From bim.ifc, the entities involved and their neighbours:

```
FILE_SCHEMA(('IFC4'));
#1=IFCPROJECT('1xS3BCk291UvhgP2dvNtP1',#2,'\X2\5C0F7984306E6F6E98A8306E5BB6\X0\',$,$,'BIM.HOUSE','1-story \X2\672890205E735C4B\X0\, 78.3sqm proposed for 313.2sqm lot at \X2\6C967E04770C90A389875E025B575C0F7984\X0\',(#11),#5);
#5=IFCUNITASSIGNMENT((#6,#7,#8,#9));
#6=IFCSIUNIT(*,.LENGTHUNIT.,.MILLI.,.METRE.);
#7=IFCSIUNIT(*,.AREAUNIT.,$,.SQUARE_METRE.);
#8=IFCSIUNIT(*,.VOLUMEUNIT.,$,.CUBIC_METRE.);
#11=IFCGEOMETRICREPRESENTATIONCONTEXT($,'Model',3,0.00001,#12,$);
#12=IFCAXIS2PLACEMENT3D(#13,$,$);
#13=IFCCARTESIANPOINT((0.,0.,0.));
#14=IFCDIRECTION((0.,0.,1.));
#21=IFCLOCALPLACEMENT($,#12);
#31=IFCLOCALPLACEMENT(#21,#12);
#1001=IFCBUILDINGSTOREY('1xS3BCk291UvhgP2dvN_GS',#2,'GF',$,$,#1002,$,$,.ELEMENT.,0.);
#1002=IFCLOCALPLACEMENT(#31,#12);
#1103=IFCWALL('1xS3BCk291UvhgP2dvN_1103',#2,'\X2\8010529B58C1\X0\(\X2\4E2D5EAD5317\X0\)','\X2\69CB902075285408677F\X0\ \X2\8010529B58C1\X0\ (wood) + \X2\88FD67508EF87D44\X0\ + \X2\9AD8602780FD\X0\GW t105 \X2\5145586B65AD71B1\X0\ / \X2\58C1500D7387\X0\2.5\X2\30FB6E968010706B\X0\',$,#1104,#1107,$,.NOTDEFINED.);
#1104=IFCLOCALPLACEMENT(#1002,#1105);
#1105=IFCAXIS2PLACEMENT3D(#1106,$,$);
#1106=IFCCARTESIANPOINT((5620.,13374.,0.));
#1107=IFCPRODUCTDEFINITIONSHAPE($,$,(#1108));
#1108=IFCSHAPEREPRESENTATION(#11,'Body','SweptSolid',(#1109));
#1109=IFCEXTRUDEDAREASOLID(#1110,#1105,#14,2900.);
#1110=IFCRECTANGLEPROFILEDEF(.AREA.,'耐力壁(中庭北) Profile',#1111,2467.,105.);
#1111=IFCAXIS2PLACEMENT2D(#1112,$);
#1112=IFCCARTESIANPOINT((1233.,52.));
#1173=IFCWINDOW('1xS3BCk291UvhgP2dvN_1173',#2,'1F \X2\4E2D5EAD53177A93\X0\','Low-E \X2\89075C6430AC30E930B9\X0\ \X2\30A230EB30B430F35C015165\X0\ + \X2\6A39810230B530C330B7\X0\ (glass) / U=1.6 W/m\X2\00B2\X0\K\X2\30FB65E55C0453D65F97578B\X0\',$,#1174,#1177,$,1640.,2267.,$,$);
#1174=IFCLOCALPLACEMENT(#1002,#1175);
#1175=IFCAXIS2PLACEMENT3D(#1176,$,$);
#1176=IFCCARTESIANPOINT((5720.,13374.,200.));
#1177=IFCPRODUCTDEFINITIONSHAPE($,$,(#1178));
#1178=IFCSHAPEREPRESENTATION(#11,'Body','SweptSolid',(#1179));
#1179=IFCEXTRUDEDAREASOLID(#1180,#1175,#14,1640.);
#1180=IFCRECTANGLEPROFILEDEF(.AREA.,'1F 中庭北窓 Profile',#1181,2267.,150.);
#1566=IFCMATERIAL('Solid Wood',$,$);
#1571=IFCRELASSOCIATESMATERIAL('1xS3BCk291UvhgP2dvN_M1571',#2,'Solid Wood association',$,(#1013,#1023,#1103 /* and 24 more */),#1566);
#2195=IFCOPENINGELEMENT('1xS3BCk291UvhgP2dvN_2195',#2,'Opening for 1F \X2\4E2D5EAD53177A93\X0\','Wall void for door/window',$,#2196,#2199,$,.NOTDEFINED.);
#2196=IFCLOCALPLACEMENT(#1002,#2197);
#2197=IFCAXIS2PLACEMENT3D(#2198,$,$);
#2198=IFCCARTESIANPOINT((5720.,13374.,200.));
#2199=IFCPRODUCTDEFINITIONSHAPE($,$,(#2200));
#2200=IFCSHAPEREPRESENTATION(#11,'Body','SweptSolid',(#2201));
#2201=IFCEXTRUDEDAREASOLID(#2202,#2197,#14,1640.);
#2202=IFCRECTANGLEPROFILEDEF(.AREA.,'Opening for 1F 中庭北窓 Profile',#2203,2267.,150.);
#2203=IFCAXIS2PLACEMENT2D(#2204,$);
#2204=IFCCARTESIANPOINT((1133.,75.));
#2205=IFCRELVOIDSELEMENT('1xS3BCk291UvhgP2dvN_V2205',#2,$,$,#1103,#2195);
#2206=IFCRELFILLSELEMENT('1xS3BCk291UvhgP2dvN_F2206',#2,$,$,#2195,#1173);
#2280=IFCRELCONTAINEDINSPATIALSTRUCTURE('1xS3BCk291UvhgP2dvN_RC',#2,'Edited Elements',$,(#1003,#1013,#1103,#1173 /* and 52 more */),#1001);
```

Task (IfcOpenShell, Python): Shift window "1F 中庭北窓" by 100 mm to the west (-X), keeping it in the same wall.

```python
import ifcopenshell
import ifcopenshell.api.geometry
import ifcopenshell.util.placement

model = ifcopenshell.open("bim.ifc")

window = model.by_id(1173)
opening = window.FillsVoids[0].RelatingOpeningElement
wall = opening.VoidsElements[0].RelatingBuildingElement

wall_matrix = ifcopenshell.util.placement.get_local_placement(wall.ObjectPlacement)
shift = wall_matrix[:3, 0] * -100.0
before = ifcopenshell.util.placement.get_local_placement(window.ObjectPlacement)[:3, 3].copy()

# The window is not placed relative to its opening, so move both.
for product in (opening, window):
    matrix = ifcopenshell.util.placement.get_local_placement(product.ObjectPlacement)
    matrix[:3, 3] += shift
    ifcopenshell.api.geometry.edit_object_placement(model, product=product, matrix=matrix, is_si=False)

after = ifcopenshell.util.placement.get_local_placement(window.ObjectPlacement)[:3, 3]
print("window moved by", (after - before).round(3) + 0.0)

model.write("bim_v2.ifc")
```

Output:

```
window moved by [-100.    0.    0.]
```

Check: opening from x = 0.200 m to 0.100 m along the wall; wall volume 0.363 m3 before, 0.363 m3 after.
